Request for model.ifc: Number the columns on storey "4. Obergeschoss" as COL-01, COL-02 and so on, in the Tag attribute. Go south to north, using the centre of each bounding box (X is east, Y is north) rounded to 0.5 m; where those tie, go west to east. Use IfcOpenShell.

First a look at what the model holds.

```python
import ifcopenshell
import ifcopenshell.util.element
import ifcopenshell.util.placement

model = ifcopenshell.open("model.ifc")
print(model.schema)
storey = next(s for s in model.by_type("IfcBuildingStorey") if s.Name == "4. Obergeschoss")
columns = [e for e in ifcopenshell.util.element.get_decomposition(storey) if e.is_a("IfcColumn")]
for e in sorted(columns, key=lambda e: e.id()):
    origin = ifcopenshell.util.placement.get_local_placement(e.ObjectPlacement)[:3, 3]
    print(e.id(), e.Tag, e.Name, origin.round(2) + 0.0, sep=" | ")
```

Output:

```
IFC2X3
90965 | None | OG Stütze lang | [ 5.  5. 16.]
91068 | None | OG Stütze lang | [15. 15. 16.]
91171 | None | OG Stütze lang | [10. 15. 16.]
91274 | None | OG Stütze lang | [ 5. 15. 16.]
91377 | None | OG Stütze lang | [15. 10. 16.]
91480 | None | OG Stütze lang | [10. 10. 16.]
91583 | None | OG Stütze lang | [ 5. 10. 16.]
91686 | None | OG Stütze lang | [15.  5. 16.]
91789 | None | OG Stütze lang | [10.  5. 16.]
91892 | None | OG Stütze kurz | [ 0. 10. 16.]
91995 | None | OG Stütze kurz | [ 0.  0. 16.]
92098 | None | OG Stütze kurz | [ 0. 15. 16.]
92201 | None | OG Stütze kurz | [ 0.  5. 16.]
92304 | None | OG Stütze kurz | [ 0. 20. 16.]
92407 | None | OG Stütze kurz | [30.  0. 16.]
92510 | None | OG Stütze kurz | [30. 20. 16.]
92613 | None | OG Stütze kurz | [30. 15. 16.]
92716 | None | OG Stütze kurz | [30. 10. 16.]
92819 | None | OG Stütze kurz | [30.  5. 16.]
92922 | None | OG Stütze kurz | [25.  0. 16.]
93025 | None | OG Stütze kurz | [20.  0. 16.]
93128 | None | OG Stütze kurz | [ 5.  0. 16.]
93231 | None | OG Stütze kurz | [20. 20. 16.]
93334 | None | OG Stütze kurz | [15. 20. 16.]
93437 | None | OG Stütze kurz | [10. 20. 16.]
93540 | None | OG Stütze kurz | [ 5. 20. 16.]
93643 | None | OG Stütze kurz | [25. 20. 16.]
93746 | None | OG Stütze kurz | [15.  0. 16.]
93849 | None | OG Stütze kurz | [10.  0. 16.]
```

```python
import ifcopenshell
import ifcopenshell.geom
import ifcopenshell.util.element
import ifcopenshell.util.shape

model = ifcopenshell.open("model.ifc")
settings = ifcopenshell.geom.settings()
settings.set("use-world-coords", True)


def centre(element):
    shape = ifcopenshell.geom.create_shape(settings, element)
    return ifcopenshell.util.shape.get_bbox_centroid(shape.geometry)


storey = next(s for s in model.by_type("IfcBuildingStorey") if s.Name == "4. Obergeschoss")
columns = [e for e in ifcopenshell.util.element.get_decomposition(storey) if e.is_a("IfcColumn")]

# Insertion points can sit at a corner or the storey origin, so sort by the geometry (in metres).
centres = {e: centre(e) for e in columns}
columns.sort(key=lambda e: (round(centres[e][1] / 0.5), centres[e][0]))

for i, e in enumerate(columns, start=1):
    number = f"COL-{i:02d}"
    e.Tag = number
    print(e.id(), number)

model.write("model_updated.ifc")
```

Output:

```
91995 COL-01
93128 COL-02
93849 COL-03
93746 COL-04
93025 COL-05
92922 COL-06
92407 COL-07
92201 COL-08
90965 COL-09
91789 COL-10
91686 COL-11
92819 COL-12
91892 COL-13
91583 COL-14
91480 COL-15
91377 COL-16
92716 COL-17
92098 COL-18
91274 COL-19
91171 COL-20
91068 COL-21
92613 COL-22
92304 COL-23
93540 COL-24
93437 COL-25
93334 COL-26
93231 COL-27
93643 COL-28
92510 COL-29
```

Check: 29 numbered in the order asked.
